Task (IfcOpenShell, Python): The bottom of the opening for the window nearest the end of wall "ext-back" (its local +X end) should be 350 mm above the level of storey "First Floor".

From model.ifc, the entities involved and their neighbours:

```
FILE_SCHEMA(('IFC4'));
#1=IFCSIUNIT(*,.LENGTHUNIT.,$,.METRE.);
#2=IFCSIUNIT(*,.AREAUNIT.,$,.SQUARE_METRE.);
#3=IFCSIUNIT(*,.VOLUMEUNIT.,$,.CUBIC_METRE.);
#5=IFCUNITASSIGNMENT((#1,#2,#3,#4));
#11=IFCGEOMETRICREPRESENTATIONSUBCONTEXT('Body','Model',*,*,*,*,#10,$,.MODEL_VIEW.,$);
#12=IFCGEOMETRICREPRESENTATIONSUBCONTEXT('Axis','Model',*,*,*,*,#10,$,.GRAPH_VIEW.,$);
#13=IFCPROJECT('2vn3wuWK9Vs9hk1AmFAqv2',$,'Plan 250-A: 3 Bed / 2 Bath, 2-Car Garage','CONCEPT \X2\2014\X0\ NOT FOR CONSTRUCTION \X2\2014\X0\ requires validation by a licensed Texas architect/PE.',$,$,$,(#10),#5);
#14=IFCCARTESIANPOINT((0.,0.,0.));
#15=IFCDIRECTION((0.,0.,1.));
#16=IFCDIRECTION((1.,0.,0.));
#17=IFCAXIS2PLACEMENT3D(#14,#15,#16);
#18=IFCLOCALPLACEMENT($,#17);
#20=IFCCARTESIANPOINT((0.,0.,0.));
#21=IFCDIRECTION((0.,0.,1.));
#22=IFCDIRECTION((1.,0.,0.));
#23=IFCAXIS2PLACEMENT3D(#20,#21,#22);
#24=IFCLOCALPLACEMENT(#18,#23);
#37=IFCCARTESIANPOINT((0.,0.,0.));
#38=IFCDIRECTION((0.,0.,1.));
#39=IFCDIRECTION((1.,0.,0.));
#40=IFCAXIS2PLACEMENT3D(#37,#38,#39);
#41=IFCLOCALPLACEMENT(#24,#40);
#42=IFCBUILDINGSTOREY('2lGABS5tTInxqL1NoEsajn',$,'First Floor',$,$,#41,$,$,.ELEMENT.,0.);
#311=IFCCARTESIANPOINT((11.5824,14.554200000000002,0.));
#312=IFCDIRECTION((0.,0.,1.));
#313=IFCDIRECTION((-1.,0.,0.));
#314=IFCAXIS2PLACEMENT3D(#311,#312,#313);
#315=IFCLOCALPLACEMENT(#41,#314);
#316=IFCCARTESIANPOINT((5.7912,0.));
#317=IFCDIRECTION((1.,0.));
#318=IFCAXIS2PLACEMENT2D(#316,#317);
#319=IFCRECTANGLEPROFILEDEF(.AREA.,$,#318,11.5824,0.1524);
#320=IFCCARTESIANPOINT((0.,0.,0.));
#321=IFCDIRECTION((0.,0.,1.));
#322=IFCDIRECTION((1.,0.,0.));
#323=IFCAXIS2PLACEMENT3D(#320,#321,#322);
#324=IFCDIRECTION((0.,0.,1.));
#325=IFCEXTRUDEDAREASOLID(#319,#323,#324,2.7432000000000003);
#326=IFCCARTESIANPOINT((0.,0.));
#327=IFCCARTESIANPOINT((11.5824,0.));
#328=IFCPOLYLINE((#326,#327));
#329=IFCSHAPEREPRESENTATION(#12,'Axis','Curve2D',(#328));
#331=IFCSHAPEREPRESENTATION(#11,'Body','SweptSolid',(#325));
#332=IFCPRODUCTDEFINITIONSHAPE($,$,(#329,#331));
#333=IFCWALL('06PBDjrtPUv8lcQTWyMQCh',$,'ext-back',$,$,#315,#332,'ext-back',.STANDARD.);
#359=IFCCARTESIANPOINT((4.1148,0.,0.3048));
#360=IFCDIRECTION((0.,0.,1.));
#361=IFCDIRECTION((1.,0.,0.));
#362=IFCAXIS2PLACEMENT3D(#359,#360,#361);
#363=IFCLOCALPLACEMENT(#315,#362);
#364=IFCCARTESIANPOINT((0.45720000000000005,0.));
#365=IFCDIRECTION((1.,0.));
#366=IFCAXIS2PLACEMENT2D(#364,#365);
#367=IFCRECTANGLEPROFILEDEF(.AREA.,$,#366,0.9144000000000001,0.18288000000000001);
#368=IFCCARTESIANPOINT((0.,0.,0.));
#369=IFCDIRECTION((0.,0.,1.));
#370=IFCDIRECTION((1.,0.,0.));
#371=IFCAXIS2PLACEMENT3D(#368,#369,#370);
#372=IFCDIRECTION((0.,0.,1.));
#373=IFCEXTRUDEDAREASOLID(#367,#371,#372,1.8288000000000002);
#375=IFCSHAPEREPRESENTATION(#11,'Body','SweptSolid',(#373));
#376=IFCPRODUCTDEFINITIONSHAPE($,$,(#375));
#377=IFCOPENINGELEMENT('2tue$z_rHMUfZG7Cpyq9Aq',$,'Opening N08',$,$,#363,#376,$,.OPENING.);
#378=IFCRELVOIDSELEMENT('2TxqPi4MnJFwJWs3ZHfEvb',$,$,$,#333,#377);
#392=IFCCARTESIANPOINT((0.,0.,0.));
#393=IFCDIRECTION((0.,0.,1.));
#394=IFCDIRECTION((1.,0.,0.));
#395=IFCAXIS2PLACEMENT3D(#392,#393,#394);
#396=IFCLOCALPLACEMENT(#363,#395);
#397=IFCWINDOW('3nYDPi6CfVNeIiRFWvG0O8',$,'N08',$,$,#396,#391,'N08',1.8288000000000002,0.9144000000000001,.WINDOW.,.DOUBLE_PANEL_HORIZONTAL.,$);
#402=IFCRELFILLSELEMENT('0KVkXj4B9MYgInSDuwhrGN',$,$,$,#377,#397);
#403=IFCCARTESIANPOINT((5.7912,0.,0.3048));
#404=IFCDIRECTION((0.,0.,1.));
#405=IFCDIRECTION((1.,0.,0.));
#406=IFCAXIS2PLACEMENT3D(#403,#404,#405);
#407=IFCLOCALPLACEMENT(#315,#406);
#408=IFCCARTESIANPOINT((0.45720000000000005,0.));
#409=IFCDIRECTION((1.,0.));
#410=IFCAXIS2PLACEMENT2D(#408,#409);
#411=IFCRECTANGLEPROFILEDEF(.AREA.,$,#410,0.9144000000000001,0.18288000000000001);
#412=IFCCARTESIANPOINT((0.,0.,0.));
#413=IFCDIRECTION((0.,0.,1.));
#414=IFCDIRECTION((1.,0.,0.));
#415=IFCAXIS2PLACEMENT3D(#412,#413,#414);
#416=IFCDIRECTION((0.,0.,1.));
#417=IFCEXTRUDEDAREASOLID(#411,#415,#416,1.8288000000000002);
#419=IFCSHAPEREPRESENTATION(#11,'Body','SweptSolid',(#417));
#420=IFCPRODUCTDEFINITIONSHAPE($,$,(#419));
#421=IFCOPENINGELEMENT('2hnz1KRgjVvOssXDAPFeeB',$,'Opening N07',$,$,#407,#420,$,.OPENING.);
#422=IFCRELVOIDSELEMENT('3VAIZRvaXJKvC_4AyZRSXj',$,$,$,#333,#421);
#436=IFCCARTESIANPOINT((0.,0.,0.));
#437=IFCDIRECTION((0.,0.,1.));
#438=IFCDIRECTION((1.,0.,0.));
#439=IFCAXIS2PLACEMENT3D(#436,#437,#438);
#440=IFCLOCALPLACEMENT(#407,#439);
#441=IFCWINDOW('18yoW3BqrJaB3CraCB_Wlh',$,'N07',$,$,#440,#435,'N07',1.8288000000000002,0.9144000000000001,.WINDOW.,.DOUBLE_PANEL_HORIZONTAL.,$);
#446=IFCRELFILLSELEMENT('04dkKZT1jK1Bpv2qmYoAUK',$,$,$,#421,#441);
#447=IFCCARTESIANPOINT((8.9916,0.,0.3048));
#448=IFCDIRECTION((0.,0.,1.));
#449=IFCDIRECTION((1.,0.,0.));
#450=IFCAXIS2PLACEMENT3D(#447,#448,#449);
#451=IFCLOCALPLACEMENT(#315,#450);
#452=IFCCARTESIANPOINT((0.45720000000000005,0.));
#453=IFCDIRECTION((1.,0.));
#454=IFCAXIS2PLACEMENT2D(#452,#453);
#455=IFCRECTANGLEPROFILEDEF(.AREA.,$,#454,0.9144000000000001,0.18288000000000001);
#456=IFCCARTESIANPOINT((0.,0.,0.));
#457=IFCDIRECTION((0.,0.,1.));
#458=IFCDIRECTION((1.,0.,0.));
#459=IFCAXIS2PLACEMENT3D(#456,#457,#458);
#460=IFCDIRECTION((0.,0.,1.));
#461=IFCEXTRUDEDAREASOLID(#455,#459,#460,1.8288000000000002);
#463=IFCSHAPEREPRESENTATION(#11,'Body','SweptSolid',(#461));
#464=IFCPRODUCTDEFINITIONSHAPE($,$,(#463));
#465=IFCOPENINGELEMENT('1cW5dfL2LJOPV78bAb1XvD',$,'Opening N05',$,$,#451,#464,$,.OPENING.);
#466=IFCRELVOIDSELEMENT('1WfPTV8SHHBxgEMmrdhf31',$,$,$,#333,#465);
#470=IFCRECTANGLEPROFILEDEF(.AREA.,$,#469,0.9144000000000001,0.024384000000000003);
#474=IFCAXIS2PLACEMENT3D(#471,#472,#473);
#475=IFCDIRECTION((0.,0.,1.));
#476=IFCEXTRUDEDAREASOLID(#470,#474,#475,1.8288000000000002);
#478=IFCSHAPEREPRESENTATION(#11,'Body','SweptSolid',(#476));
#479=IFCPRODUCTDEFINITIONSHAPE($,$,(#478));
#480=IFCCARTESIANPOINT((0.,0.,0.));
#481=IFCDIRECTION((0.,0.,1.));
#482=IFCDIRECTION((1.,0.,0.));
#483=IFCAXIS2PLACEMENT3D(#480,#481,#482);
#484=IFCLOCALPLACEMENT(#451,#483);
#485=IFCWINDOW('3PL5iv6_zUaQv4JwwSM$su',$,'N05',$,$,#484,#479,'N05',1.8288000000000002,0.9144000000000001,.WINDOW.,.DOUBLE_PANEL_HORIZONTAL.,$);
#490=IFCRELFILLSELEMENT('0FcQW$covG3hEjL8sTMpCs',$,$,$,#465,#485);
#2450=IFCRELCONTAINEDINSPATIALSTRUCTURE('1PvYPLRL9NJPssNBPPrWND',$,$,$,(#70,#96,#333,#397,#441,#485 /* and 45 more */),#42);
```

```python
import numpy as np
import ifcopenshell
import ifcopenshell.api.geometry
import ifcopenshell.geom
import ifcopenshell.util.element
import ifcopenshell.util.placement
import ifcopenshell.util.shape
import ifcopenshell.util.unit

model = ifcopenshell.open("model.ifc")
unit_scale = ifcopenshell.util.unit.calculate_unit_scale(model)

window = model.by_guid("3PL5iv6_zUaQv4JwwSM$su")
opening = window.FillsVoids[0].RelatingOpeningElement
storey = ifcopenshell.util.element.get_container(window, ifc_class="IfcBuildingStorey")
level = ifcopenshell.util.placement.get_local_placement(storey.ObjectPlacement)[2, 3]

# The opening's origin need not be at the sill, so measure its lowest point.
shape = ifcopenshell.geom.create_shape(ifcopenshell.geom.settings(), opening)
bottom = ifcopenshell.util.shape.get_shape_bottom_elevation(shape, shape.geometry) / unit_scale
dz = level + 0.35 / unit_scale - bottom

shift = np.array([0.0, 0.0, dz])
# The window is placed relative to its opening, so it follows when the opening moves.
matrix = ifcopenshell.util.placement.get_local_placement(opening.ObjectPlacement)
matrix[:3, 3] += shift
ifcopenshell.api.geometry.edit_object_placement(
    model, product=opening, matrix=matrix, is_si=False, should_transform_children=True
)

print(f"moved by {dz * unit_scale:+.3f} m")

model.write("model_edited.ifc")
```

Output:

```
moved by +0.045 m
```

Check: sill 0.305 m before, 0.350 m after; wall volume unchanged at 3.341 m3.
